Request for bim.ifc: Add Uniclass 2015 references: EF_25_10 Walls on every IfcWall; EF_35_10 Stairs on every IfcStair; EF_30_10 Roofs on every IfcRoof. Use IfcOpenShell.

First a look at what the model holds.

```python
import ifcopenshell

model = ifcopenshell.open("bim.ifc")
print(model.schema)
print("classifications:", [c.Name for c in model.by_type("IfcClassification")])
for ifc_class in ("IfcDoor", "IfcRoof", "IfcStair", "IfcWall", "IfcWindow"):
    print(ifc_class, len(model.by_type(ifc_class)))
```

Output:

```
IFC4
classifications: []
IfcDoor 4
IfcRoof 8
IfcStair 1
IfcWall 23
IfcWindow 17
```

```python
import ifcopenshell
import ifcopenshell.api.classification

model = ifcopenshell.open("bim.ifc")

system = ifcopenshell.api.classification.add_classification(model, classification="Uniclass 2015")

codes = {
    "IfcWall": ("EF_25_10", "Walls"),
    "IfcStair": ("EF_35_10", "Stairs"),
    "IfcRoof": ("EF_30_10", "Roofs"),
}
for ifc_class, (code, name) in codes.items():
    products = model.by_type(ifc_class)
    ifcopenshell.api.classification.add_reference(
        model, products=products, classification=system, identification=code, name=name
    )
    print(code, len(products))

model.write("bim_edited.ifc")
```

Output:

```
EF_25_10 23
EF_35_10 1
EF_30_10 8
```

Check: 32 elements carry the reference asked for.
